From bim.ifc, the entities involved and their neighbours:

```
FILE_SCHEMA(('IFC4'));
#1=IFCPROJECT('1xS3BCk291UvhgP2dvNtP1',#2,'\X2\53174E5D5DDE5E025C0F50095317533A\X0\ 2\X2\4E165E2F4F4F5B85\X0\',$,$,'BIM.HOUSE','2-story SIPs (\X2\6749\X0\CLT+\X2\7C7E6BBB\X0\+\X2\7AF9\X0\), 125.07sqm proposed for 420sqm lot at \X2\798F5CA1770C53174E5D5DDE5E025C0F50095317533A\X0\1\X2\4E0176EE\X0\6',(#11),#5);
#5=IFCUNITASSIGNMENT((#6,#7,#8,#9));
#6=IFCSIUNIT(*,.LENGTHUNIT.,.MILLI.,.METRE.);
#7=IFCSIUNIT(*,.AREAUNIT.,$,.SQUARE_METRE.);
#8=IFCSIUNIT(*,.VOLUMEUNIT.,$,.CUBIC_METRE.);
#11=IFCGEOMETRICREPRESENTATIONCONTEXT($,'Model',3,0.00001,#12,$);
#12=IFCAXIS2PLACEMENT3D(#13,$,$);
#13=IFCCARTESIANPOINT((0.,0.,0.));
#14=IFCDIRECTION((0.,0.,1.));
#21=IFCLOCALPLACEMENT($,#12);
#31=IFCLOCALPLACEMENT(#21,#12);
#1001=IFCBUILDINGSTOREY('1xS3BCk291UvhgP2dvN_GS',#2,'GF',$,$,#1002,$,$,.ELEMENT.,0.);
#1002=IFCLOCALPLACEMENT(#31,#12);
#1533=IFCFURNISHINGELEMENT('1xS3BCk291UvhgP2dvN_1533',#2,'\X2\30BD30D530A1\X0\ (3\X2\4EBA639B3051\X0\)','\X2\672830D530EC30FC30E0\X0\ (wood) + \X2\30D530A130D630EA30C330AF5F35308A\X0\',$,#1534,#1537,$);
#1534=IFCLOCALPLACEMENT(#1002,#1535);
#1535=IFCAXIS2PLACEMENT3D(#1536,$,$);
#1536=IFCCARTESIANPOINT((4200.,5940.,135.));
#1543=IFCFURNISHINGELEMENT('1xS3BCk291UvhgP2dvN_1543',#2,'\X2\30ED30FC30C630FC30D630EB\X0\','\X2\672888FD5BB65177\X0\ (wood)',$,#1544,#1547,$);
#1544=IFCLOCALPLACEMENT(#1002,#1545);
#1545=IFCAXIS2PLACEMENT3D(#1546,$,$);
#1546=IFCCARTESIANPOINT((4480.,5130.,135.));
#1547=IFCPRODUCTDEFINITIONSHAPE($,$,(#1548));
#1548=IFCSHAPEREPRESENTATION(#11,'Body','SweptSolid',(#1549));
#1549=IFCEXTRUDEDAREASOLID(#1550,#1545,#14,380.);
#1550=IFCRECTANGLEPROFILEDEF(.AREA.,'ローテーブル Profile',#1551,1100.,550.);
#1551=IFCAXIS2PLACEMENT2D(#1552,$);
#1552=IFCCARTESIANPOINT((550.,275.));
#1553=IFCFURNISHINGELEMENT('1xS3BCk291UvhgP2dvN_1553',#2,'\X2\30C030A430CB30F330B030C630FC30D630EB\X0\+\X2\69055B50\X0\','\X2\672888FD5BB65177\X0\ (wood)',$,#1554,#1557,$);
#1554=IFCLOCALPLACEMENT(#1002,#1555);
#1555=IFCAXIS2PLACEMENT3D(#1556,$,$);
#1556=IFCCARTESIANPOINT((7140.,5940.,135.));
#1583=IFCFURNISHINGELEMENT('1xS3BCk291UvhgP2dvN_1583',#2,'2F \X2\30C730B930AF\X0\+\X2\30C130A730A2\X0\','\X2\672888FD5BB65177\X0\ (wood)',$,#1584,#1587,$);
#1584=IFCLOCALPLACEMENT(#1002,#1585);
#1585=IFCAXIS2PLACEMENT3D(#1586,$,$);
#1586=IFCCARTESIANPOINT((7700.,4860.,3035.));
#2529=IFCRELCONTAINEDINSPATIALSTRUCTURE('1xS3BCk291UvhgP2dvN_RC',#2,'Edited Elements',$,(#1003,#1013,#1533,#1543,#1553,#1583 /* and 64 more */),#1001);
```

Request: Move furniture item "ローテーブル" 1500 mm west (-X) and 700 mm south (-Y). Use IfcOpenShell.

```python
import ifcopenshell
import ifcopenshell.api.geometry
import ifcopenshell.util.placement
import ifcopenshell.util.unit

model = ifcopenshell.open("bim.ifc")
unit_scale = ifcopenshell.util.unit.calculate_unit_scale(model)

item = model.by_guid("1xS3BCk291UvhgP2dvN_1543")
matrix = ifcopenshell.util.placement.get_local_placement(item.ObjectPlacement)
matrix[0, 3] -= 1.5 / unit_scale
matrix[1, 3] -= 0.7 / unit_scale
ifcopenshell.api.geometry.edit_object_placement(model, product=item, matrix=matrix, is_si=False)

print(ifcopenshell.util.placement.get_local_placement(item.ObjectPlacement).round(3) + 0.0)

model.write("bim_edited.ifc")
```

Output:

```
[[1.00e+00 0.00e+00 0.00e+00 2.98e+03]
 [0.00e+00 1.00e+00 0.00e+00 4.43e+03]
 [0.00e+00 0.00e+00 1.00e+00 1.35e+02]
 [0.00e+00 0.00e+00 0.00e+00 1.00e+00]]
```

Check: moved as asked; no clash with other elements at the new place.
